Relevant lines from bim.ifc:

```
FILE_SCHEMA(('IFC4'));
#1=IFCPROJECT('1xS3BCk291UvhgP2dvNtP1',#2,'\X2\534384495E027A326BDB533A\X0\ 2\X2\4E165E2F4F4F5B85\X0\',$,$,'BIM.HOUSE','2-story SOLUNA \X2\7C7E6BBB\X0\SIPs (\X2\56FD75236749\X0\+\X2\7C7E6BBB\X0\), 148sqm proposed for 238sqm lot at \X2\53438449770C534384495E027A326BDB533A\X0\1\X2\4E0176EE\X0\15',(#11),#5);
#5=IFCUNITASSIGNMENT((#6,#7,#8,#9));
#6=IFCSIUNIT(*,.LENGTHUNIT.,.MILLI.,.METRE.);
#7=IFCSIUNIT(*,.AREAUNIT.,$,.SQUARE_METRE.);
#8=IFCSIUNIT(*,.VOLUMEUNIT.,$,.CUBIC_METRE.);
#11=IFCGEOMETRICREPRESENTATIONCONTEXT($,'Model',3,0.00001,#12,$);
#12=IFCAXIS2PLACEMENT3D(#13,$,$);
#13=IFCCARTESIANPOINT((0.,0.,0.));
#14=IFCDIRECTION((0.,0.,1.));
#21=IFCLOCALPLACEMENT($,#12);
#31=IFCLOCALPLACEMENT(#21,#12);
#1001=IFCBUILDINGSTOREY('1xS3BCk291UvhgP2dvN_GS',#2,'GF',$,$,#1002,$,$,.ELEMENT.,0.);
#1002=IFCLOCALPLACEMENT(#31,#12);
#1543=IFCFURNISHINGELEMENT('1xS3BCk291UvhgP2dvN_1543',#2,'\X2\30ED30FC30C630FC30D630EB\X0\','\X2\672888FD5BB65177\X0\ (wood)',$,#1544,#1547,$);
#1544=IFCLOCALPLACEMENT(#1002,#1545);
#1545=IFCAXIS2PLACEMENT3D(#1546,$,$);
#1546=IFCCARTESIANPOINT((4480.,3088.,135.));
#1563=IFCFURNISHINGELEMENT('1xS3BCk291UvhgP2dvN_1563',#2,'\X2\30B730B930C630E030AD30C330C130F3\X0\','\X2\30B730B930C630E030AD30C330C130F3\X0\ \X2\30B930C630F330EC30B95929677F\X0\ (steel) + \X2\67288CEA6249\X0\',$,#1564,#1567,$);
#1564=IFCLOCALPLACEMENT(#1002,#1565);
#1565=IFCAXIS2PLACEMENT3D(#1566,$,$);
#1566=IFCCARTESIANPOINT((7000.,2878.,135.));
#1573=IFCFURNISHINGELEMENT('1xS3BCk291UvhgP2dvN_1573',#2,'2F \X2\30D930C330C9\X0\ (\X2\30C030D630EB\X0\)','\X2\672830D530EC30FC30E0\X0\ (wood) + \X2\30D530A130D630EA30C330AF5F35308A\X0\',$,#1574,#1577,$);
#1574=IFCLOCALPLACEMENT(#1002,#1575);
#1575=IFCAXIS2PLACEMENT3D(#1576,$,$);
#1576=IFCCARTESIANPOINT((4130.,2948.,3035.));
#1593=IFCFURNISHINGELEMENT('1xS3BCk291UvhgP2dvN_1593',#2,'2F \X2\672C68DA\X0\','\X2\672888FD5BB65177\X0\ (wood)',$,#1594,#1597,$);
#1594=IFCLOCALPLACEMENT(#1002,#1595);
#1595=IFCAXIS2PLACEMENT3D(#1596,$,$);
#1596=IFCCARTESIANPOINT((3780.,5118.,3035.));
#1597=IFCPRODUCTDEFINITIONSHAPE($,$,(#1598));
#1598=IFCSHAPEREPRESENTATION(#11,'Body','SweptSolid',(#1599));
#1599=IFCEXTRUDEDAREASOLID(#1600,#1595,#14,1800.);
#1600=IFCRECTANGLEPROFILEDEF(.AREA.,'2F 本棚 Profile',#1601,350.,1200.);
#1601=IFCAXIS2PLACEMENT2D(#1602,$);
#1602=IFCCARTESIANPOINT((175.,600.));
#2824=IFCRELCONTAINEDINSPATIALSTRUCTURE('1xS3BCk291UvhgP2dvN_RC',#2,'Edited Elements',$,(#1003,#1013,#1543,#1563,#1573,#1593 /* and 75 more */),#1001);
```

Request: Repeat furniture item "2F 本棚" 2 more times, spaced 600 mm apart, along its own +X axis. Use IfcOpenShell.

```python
import ifcopenshell
import ifcopenshell.api.geometry
import ifcopenshell.api.root
import ifcopenshell.util.element
import ifcopenshell.util.placement
import ifcopenshell.util.unit

model = ifcopenshell.open("bim.ifc")
unit_scale = ifcopenshell.util.unit.calculate_unit_scale(model)


def reuse_history(source, copy):
    """copy_class also copies each property set's owner history, people and application; keep the originals."""
    for rel in copy.IsDefinedBy:
        if rel.is_a("IfcRelDefinesByProperties") and (history := rel.RelatingPropertyDefinition.OwnerHistory):
            rel.RelatingPropertyDefinition.OwnerHistory = source.OwnerHistory
            ifcopenshell.util.element.remove_deep2(model, history)


source = model.by_guid("1xS3BCk291UvhgP2dvN_1593")
base = ifcopenshell.util.placement.get_local_placement(source.ObjectPlacement)
step = base[:3, 0] * 0.6 / unit_scale

for i in range(1, 3):
    copy = ifcopenshell.api.root.copy_class(model, product=source)
    copy.Representation = ifcopenshell.util.element.copy_deep(
        model, source.Representation, exclude=["IfcGeometricRepresentationContext", "IfcRepresentationMap"]
    )
    reuse_history(source, copy)
    matrix = base.copy()
    matrix[:3, 3] += i * step
    print("added at", matrix[:3, 3].round(3) + 0.0)
    ifcopenshell.api.geometry.edit_object_placement(model, product=copy, matrix=matrix, is_si=False)

model.write("bim_edited.ifc")
```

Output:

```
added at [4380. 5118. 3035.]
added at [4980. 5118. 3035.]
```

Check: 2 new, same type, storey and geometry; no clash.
